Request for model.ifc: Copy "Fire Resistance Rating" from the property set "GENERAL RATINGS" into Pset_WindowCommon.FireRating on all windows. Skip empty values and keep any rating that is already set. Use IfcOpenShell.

First a look at what the model holds.

```python
import ifcopenshell
import ifcopenshell.util.element

model = ifcopenshell.open("model.ifc")
print(model.schema)
windows = model.by_type("IfcWindow")
print(len(windows), "windows")
for e in windows[:8]:
    source = ifcopenshell.util.element.get_pset(e, "GENERAL RATINGS", "Fire Resistance Rating")
    target = ifcopenshell.util.element.get_pset(e, "Pset_WindowCommon", "FireRating")
    print(e.id(), repr(source), repr(target), sep=" | ")
```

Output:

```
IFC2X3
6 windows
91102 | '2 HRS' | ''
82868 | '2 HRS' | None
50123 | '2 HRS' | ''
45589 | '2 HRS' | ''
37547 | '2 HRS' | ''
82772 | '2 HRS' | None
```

```python
import ifcopenshell
import ifcopenshell.api.pset
import ifcopenshell.util.element

model = ifcopenshell.open("model.ifc")

count = 0
for e in model.by_type("IfcWindow"):
    value = ifcopenshell.util.element.get_pset(e, "GENERAL RATINGS", "Fire Resistance Rating")
    current = ifcopenshell.util.element.get_pset(e, "Pset_WindowCommon", "FireRating")
    if not value or not value.strip() or current:
        continue
    # add_pset returns the element's existing set when there is one.
    pset = ifcopenshell.api.pset.add_pset(model, product=e, name="Pset_WindowCommon")
    ifcopenshell.api.pset.edit_pset(model, pset=pset, properties={"FireRating": value})
    count += 1

print(count, "windows updated")

model.write("model_rev.ifc")
```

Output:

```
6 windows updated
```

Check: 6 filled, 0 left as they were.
